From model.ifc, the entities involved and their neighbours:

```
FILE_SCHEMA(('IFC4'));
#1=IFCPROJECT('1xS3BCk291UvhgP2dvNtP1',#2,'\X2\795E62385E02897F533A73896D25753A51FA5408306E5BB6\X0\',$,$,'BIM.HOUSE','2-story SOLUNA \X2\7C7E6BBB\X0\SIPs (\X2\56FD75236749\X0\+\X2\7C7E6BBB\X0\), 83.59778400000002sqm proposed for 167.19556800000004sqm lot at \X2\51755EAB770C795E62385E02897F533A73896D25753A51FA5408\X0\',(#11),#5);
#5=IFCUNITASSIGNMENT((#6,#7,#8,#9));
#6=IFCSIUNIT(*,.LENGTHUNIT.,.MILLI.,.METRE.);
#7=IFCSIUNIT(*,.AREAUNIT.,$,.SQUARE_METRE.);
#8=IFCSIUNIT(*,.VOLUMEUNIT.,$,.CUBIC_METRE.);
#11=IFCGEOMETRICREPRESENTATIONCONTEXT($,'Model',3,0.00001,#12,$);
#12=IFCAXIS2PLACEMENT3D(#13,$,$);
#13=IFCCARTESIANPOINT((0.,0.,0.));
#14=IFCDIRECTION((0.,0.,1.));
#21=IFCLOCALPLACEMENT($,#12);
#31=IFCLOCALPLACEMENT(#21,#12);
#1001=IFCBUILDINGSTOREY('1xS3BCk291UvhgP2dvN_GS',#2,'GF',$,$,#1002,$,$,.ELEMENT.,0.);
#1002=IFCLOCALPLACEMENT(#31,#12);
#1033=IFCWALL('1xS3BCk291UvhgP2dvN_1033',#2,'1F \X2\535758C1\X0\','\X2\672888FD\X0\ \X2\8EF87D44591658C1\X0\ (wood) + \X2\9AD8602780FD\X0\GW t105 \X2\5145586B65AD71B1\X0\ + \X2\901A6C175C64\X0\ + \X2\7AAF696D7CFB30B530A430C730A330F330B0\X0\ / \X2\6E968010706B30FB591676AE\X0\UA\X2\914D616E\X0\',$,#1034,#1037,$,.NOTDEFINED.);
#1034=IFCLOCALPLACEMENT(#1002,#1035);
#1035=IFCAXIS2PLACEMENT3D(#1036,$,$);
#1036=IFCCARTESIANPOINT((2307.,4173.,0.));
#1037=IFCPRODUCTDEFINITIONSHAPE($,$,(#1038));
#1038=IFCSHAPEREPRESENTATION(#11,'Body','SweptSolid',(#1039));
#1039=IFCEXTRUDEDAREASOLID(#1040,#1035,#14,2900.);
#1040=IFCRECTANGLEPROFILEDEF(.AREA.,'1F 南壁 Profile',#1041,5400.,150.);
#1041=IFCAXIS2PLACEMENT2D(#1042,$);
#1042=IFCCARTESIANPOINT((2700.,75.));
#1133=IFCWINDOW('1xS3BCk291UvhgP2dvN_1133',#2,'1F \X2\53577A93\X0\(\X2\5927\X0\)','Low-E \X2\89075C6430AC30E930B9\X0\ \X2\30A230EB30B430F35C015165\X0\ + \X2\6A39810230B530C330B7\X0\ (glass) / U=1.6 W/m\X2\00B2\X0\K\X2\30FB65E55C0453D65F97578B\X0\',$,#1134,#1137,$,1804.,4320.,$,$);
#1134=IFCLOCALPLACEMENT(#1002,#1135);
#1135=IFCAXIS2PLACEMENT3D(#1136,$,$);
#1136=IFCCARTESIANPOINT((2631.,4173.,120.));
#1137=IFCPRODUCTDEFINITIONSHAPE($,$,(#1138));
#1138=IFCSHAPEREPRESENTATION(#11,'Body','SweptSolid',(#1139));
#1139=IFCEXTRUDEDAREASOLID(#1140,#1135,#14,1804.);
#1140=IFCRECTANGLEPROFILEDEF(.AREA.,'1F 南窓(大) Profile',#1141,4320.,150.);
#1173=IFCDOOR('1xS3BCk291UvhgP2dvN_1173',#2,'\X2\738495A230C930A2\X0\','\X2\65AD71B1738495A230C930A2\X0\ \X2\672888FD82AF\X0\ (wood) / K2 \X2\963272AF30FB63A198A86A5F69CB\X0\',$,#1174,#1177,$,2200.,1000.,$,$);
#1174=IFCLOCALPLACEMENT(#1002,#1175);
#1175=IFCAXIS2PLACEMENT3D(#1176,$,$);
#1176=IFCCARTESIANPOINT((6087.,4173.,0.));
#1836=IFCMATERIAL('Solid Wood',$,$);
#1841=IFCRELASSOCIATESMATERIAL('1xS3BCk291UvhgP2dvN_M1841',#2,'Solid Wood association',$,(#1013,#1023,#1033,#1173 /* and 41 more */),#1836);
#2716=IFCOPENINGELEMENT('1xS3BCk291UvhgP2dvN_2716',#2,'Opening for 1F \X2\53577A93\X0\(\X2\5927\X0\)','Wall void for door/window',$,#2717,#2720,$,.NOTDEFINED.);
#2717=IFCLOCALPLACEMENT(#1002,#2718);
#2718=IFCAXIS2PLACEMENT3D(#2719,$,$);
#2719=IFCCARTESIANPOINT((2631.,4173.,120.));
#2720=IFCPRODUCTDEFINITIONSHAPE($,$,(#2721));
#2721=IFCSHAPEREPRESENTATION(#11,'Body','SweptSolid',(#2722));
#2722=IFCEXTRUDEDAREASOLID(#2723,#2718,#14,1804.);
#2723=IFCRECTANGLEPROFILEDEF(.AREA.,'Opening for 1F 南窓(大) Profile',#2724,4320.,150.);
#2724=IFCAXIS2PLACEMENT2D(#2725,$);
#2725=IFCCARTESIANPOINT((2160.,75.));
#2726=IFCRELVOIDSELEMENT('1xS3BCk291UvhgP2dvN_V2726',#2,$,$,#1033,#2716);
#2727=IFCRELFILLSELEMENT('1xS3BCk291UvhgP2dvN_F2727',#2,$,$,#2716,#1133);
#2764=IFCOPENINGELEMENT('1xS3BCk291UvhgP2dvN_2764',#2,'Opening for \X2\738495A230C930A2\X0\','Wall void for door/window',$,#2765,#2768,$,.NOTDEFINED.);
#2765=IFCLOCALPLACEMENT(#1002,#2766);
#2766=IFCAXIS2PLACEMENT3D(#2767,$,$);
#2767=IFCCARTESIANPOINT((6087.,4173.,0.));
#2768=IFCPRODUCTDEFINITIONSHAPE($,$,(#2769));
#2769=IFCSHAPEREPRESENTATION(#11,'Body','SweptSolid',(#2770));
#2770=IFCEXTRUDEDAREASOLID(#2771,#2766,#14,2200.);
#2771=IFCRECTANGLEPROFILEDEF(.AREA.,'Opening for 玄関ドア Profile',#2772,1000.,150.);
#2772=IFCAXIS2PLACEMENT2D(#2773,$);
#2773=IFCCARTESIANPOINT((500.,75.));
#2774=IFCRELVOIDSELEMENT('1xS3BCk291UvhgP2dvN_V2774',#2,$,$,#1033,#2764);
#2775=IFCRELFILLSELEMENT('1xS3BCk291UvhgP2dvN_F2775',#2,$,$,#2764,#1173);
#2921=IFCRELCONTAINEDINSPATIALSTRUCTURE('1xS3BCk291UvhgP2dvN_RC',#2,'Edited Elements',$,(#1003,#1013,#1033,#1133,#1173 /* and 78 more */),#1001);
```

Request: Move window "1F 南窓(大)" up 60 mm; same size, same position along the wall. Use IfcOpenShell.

```python
import numpy as np
import ifcopenshell
import ifcopenshell.api.geometry
import ifcopenshell.util.placement
import ifcopenshell.util.unit

model = ifcopenshell.open("model.ifc")
unit_scale = ifcopenshell.util.unit.calculate_unit_scale(model)

window = model.by_id(1133)
opening = window.FillsVoids[0].RelatingOpeningElement
dz = 0.06 / unit_scale

shift = np.array([0.0, 0.0, dz])
# The window is not placed relative to its opening, so move both.
for product in (opening, window):
    matrix = ifcopenshell.util.placement.get_local_placement(product.ObjectPlacement)
    matrix[:3, 3] += shift
    ifcopenshell.api.geometry.edit_object_placement(model, product=product, matrix=matrix, is_si=False)

print(f"moved by {dz * unit_scale:+.3f} m")

model.write("model_v2.ifc")
```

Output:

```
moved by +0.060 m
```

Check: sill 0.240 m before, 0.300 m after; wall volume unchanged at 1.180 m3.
